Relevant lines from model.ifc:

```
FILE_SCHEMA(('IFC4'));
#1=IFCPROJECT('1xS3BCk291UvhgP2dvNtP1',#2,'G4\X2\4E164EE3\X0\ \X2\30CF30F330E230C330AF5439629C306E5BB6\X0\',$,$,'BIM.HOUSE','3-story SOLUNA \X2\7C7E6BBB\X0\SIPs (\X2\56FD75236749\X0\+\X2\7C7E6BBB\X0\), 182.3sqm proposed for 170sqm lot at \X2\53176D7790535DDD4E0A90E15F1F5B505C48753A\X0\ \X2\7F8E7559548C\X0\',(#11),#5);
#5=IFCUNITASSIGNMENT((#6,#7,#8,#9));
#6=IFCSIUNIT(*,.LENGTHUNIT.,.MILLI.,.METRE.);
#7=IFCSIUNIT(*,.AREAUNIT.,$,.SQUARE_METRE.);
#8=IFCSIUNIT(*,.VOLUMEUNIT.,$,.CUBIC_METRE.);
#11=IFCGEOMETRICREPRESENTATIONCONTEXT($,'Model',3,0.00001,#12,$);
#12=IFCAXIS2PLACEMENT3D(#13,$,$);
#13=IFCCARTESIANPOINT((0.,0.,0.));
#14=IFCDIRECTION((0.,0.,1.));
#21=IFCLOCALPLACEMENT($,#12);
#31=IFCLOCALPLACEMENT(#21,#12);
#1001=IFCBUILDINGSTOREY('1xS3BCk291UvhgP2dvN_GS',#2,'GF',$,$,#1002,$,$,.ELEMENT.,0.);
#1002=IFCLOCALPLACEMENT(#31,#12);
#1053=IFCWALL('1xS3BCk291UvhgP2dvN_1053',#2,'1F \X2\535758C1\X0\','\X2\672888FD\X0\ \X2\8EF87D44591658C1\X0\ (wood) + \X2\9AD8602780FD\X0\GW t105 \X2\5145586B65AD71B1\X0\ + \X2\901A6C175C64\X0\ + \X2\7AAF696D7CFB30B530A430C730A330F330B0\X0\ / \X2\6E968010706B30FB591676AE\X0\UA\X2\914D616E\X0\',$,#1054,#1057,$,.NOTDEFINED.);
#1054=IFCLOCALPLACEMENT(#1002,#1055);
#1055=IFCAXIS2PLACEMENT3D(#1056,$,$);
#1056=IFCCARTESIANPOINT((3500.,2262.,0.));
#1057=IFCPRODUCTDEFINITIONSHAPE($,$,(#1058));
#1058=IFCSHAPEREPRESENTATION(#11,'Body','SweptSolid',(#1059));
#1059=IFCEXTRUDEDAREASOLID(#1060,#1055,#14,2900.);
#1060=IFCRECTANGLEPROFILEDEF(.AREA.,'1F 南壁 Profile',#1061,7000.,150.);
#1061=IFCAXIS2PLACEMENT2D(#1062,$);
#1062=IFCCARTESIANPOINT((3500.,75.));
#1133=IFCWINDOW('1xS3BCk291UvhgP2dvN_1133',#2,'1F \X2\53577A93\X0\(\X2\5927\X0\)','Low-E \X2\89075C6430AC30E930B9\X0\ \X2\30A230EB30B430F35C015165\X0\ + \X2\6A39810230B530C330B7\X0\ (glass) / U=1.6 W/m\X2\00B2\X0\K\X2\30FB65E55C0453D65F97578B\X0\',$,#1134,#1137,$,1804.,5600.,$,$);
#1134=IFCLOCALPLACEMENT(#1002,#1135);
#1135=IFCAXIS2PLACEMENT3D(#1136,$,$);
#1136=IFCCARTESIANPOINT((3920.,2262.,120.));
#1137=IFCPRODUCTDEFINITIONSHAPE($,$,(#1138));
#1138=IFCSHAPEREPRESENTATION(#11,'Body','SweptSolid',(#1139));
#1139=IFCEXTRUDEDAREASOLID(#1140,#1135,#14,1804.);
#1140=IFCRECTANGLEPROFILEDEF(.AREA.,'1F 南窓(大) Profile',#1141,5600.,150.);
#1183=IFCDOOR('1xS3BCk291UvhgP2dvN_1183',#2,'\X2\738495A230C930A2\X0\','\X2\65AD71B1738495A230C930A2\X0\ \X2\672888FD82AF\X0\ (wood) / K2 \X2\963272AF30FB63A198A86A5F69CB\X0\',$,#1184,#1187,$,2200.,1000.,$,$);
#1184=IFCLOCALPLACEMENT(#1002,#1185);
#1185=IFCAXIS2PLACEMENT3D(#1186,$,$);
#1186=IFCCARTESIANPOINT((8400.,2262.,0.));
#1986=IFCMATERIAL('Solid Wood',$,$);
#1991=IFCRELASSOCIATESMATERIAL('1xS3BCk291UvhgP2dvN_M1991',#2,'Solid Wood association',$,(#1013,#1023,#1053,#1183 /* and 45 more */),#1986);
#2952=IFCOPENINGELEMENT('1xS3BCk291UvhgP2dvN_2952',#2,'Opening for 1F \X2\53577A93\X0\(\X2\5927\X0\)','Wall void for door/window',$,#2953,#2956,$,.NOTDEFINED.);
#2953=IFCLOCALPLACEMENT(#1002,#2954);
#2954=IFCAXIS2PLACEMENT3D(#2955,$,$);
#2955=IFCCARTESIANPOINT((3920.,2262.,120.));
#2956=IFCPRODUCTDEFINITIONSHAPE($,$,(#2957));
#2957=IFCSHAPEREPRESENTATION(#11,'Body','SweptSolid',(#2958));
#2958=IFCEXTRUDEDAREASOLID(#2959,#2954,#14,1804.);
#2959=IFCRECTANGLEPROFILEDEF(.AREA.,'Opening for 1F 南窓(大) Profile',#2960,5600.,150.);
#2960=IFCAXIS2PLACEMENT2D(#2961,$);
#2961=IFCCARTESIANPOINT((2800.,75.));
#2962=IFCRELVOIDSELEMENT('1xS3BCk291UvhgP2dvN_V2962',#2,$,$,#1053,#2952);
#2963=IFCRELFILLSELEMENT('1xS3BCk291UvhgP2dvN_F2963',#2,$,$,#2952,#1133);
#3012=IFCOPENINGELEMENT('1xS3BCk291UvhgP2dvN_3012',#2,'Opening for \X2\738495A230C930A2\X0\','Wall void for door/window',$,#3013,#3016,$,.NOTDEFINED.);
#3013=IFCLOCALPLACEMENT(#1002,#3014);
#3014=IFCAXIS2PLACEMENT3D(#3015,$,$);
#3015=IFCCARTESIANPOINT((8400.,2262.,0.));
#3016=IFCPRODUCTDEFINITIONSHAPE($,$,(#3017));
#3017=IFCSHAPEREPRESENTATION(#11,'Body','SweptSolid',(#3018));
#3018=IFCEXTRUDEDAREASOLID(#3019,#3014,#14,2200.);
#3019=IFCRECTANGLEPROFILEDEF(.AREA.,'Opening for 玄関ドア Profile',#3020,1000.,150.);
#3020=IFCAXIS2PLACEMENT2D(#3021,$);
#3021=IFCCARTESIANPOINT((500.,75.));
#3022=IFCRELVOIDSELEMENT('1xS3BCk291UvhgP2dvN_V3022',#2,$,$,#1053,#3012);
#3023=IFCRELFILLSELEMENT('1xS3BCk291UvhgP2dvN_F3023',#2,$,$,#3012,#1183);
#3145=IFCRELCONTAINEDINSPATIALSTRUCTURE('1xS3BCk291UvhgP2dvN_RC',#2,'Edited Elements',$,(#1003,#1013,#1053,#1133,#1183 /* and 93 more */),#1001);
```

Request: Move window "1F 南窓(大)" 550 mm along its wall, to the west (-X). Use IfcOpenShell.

```python
import ifcopenshell
import ifcopenshell.api.geometry
import ifcopenshell.util.placement
import ifcopenshell.util.unit

model = ifcopenshell.open("model.ifc")
unit_scale = ifcopenshell.util.unit.calculate_unit_scale(model)

window = model.by_guid("1xS3BCk291UvhgP2dvN_1133")
opening = window.FillsVoids[0].RelatingOpeningElement
wall = opening.VoidsElements[0].RelatingBuildingElement

wall_matrix = ifcopenshell.util.placement.get_local_placement(wall.ObjectPlacement)
shift = wall_matrix[:3, 0] * -0.55 / unit_scale
before = ifcopenshell.util.placement.get_local_placement(window.ObjectPlacement)[:3, 3].copy()

# The window is not placed relative to its opening, so move both.
for product in (opening, window):
    matrix = ifcopenshell.util.placement.get_local_placement(product.ObjectPlacement)
    matrix[:3, 3] += shift
    ifcopenshell.api.geometry.edit_object_placement(model, product=product, matrix=matrix, is_si=False)

after = ifcopenshell.util.placement.get_local_placement(window.ObjectPlacement)[:3, 3]
print("window moved by", (after - before).round(3) + 0.0)

model.write("model_edited.ifc")
```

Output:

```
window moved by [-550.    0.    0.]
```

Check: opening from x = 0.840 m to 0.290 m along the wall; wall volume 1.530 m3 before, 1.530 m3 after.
